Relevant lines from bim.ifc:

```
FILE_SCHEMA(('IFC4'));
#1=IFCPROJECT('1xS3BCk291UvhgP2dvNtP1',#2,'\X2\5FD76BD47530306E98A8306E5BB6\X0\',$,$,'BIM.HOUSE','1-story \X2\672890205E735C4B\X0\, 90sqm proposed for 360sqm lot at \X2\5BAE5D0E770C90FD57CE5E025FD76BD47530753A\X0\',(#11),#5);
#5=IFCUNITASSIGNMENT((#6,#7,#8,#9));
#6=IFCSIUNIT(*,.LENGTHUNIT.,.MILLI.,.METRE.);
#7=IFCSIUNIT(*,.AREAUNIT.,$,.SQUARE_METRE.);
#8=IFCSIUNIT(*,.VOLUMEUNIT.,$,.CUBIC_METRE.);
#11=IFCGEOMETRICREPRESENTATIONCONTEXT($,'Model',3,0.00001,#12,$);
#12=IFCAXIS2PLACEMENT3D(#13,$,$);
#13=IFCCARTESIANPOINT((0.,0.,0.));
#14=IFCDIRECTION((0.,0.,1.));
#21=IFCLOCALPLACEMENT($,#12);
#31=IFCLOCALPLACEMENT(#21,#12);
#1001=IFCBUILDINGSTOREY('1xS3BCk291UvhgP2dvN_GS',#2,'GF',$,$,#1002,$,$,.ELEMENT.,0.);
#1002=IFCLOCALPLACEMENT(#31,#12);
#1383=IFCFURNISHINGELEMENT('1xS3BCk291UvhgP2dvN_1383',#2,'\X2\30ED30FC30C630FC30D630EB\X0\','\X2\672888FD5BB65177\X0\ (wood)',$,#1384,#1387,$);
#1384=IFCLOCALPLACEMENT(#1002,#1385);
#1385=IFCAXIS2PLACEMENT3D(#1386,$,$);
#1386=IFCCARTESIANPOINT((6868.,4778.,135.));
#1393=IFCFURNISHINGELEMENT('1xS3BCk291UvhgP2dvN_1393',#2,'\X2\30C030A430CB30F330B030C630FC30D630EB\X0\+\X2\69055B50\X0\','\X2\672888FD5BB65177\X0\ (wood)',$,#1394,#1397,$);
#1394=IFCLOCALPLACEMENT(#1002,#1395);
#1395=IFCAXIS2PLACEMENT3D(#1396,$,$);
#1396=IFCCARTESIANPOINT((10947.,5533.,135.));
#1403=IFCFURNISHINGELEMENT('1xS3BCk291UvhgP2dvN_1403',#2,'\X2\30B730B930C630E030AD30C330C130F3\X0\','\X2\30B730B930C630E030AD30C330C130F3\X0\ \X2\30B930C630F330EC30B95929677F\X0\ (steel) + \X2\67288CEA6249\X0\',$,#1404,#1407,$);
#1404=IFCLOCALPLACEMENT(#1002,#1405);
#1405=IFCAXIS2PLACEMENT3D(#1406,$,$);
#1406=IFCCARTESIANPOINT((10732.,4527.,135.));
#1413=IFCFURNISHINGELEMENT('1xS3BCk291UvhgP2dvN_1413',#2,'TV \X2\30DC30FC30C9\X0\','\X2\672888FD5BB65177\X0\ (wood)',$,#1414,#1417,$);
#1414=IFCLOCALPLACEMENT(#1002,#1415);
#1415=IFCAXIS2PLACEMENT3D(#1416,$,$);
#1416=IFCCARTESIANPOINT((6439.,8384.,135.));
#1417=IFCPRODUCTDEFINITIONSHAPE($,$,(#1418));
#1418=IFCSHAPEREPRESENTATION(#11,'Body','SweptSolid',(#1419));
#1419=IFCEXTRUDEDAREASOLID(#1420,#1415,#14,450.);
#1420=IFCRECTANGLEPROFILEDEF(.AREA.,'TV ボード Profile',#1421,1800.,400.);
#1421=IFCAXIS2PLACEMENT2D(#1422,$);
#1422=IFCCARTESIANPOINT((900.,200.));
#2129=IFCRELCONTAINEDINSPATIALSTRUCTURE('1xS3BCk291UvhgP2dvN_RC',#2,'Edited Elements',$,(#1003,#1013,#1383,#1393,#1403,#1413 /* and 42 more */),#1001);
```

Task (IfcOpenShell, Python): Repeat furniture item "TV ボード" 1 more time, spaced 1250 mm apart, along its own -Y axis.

```python
import ifcopenshell
import ifcopenshell.api.geometry
import ifcopenshell.api.root
import ifcopenshell.util.element
import ifcopenshell.util.placement

model = ifcopenshell.open("bim.ifc")


def reuse_history(source, copy):
    """copy_class also copies each property set's owner history, people and application; keep the originals."""
    for rel in copy.IsDefinedBy:
        if rel.is_a("IfcRelDefinesByProperties") and (history := rel.RelatingPropertyDefinition.OwnerHistory):
            rel.RelatingPropertyDefinition.OwnerHistory = source.OwnerHistory
            ifcopenshell.util.element.remove_deep2(model, history)


source = model.by_id(1413)
base = ifcopenshell.util.placement.get_local_placement(source.ObjectPlacement)
step = -base[:3, 1] * 1250.0

for i in range(1, 2):
    copy = ifcopenshell.api.root.copy_class(model, product=source)
    copy.Representation = ifcopenshell.util.element.copy_deep(
        model, source.Representation, exclude=["IfcGeometricRepresentationContext", "IfcRepresentationMap"]
    )
    reuse_history(source, copy)
    matrix = base.copy()
    matrix[:3, 3] += i * step
    print("added at", matrix[:3, 3].round(3) + 0.0)
    ifcopenshell.api.geometry.edit_object_placement(model, product=copy, matrix=matrix, is_si=False)

model.write("bim_edited.ifc")
```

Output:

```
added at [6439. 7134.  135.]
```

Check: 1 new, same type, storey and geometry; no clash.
